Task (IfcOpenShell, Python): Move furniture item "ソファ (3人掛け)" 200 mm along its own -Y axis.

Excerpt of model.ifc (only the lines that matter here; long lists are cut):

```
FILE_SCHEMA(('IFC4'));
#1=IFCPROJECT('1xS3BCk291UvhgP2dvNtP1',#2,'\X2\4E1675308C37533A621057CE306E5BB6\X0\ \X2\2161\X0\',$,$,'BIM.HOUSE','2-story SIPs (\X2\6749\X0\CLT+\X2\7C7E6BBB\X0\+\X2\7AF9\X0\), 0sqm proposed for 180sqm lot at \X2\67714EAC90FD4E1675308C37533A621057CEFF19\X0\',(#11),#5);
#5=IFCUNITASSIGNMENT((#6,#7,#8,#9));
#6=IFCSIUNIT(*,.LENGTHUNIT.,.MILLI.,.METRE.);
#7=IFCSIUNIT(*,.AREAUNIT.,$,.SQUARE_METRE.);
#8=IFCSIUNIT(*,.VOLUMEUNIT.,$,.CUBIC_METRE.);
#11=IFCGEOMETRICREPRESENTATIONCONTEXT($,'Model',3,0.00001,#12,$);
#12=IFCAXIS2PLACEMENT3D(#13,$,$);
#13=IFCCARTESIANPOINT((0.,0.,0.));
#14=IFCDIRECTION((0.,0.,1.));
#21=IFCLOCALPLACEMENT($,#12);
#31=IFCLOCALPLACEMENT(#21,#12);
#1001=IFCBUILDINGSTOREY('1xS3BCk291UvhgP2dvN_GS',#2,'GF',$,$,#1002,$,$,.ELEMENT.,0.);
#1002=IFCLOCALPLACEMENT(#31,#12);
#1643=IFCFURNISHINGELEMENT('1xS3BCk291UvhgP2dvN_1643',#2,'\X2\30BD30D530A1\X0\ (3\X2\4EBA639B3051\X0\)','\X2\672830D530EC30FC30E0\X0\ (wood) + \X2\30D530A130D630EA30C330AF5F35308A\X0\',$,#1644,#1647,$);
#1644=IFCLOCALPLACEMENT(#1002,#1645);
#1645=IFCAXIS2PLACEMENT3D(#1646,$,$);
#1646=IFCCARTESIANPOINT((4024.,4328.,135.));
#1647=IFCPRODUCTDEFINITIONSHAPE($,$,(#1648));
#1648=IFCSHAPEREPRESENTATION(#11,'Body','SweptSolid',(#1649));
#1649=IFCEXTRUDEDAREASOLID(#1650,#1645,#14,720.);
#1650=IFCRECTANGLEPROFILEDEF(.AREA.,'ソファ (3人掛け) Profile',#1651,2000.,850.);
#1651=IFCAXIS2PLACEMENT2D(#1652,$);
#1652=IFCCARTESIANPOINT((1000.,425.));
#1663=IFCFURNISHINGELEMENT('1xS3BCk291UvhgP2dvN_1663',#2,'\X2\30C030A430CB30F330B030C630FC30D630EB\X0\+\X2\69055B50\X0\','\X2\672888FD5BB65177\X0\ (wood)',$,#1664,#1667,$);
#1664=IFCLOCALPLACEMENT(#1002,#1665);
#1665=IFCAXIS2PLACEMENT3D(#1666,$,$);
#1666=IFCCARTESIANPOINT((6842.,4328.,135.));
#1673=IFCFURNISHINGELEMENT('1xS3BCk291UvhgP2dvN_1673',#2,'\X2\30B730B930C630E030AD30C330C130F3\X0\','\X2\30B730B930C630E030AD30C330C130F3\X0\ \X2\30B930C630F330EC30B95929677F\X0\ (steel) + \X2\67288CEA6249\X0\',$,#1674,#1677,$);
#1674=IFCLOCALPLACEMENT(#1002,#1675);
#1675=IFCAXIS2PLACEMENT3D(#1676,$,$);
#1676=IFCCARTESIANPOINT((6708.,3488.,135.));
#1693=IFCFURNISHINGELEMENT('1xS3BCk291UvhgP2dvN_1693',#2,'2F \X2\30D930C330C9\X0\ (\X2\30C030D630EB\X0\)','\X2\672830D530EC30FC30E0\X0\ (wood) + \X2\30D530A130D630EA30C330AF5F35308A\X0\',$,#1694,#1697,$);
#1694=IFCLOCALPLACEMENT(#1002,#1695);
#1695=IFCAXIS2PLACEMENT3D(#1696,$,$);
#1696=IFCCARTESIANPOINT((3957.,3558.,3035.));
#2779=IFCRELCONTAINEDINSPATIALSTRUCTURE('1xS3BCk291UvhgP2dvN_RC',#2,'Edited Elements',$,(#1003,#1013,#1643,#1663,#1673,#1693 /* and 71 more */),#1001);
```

```python
import ifcopenshell
import ifcopenshell.api.geometry
import ifcopenshell.util.placement

model = ifcopenshell.open("model.ifc")

item = model.by_id(1643)
matrix = ifcopenshell.util.placement.get_local_placement(item.ObjectPlacement)
matrix[:3, 3] -= matrix[:3, 1] * 200.0
ifcopenshell.api.geometry.edit_object_placement(model, product=item, matrix=matrix, is_si=False)

print(ifcopenshell.util.placement.get_local_placement(item.ObjectPlacement).round(3) + 0.0)

model.write("model_v2.ifc")
```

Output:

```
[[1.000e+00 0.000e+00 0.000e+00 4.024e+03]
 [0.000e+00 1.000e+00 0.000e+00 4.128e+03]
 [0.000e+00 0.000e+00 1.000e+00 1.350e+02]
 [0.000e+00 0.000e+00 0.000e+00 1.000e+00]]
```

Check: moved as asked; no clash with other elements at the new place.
